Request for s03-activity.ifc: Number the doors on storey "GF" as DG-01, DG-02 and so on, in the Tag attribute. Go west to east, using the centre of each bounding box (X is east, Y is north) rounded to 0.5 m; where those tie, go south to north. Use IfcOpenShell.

First a look at what the model holds.

```python
import ifcopenshell
import ifcopenshell.util.element
import ifcopenshell.util.placement

model = ifcopenshell.open("s03-activity.ifc")
print(model.schema)
storey = next(s for s in model.by_type("IfcBuildingStorey") if s.Name == "GF")
doors = [e for e in ifcopenshell.util.element.get_decomposition(storey) if e.is_a("IfcDoor")]
for e in sorted(doors, key=lambda e: e.id()):
    origin = ifcopenshell.util.placement.get_local_placement(e.ObjectPlacement)[:3, 3]
    print(e.id(), e.Tag, e.Name, origin.round(2) + 0.0, sep=" | ")
```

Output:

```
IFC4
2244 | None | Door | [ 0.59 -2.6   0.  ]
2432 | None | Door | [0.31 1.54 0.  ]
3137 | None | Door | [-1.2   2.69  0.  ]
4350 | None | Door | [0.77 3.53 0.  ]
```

```python
import ifcopenshell
import ifcopenshell.geom
import ifcopenshell.util.element
import ifcopenshell.util.shape

model = ifcopenshell.open("s03-activity.ifc")
settings = ifcopenshell.geom.settings()
settings.set("use-world-coords", True)


def centre(element):
    shape = ifcopenshell.geom.create_shape(settings, element)
    return ifcopenshell.util.shape.get_bbox_centroid(shape.geometry)


storey = next(s for s in model.by_type("IfcBuildingStorey") if s.Name == "GF")
doors = [e for e in ifcopenshell.util.element.get_decomposition(storey) if e.is_a("IfcDoor")]

# Insertion points can sit at a corner or the storey origin, so sort by the geometry (in metres).
centres = {e: centre(e) for e in doors}
doors.sort(key=lambda e: (round(centres[e][0] / 0.5), centres[e][1]))

for i, e in enumerate(doors, start=1):
    number = f"DG-{i:02d}"
    e.Tag = number
    print(e.id(), number)

model.write("s03-activity_edited.ifc")
```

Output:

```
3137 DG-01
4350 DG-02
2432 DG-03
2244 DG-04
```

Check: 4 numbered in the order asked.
